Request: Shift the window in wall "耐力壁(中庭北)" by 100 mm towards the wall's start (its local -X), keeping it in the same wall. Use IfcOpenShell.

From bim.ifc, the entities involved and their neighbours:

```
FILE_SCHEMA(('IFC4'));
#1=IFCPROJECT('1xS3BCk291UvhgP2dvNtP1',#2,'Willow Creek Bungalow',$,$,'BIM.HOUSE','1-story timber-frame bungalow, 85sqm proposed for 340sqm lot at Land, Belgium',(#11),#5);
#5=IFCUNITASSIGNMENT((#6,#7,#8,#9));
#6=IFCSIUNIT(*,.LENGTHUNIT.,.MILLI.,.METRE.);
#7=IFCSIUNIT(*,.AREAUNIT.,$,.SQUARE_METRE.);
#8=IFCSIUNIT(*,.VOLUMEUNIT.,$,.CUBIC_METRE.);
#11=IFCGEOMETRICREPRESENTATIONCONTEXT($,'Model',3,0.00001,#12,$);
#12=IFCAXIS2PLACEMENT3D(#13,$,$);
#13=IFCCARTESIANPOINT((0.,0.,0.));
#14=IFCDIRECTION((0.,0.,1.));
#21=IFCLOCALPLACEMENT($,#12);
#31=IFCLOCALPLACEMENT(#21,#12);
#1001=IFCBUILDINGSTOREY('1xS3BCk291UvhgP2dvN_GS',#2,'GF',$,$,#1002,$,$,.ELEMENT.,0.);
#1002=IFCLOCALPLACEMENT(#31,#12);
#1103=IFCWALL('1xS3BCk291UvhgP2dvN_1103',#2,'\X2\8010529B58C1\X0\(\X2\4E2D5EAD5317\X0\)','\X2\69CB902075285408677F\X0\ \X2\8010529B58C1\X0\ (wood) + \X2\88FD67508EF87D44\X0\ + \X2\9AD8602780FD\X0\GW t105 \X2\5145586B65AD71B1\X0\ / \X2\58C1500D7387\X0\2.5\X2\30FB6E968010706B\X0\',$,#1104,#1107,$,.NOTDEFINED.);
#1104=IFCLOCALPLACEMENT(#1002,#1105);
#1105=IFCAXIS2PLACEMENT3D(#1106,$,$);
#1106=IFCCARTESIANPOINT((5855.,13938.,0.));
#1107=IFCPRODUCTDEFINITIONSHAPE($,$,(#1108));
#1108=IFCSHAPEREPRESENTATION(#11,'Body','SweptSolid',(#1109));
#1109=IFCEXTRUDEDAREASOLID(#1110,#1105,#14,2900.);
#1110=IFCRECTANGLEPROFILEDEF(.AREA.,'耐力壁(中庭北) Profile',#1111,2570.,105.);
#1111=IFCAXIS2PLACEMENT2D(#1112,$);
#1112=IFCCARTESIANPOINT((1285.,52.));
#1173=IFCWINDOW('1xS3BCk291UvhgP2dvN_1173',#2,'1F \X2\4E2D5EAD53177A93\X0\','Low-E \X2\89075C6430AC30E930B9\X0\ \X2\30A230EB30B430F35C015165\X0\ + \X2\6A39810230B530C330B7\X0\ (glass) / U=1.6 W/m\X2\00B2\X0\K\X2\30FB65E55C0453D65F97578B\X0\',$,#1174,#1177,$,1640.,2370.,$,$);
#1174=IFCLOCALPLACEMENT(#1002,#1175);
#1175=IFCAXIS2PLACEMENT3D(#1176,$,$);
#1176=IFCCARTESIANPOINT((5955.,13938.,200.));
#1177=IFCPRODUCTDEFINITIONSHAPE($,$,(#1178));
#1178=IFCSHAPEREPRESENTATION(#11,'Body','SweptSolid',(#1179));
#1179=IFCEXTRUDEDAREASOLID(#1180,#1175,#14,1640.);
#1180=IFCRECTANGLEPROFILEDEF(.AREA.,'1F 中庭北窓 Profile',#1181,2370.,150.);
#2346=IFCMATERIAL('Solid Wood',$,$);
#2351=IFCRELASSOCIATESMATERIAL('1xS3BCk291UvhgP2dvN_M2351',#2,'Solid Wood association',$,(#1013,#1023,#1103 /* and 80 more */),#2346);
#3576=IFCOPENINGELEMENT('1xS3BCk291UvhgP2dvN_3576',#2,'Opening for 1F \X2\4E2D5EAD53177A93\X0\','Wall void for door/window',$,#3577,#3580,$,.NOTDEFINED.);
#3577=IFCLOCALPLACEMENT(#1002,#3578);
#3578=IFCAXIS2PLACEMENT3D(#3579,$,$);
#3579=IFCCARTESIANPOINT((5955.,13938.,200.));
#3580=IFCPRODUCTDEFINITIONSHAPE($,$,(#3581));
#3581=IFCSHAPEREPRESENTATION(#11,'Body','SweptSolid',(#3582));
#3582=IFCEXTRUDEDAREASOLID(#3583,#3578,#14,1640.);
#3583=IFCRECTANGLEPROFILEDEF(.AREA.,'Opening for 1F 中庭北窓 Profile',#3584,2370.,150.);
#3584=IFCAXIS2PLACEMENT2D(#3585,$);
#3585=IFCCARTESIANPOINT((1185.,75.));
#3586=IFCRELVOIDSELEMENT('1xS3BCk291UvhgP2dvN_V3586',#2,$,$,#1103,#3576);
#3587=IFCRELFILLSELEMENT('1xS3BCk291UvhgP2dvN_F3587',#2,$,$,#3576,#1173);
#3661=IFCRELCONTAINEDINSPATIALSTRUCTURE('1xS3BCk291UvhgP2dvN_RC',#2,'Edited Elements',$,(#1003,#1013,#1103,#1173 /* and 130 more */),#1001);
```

```python
import ifcopenshell
import ifcopenshell.api.geometry
import ifcopenshell.util.placement
import ifcopenshell.util.unit

model = ifcopenshell.open("bim.ifc")
unit_scale = ifcopenshell.util.unit.calculate_unit_scale(model)

window = model.by_id(1173)
opening = window.FillsVoids[0].RelatingOpeningElement
wall = opening.VoidsElements[0].RelatingBuildingElement

wall_matrix = ifcopenshell.util.placement.get_local_placement(wall.ObjectPlacement)
shift = wall_matrix[:3, 0] * -0.1 / unit_scale
before = ifcopenshell.util.placement.get_local_placement(window.ObjectPlacement)[:3, 3].copy()

# The window is not placed relative to its opening, so move both.
for product in (opening, window):
    matrix = ifcopenshell.util.placement.get_local_placement(product.ObjectPlacement)
    matrix[:3, 3] += shift
    ifcopenshell.api.geometry.edit_object_placement(model, product=product, matrix=matrix, is_si=False)

after = ifcopenshell.util.placement.get_local_placement(window.ObjectPlacement)[:3, 3]
print("window moved by", (after - before).round(3) + 0.0)

model.write("bim-out.ifc")
```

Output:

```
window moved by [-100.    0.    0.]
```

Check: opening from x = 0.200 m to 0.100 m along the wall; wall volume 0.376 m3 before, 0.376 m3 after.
